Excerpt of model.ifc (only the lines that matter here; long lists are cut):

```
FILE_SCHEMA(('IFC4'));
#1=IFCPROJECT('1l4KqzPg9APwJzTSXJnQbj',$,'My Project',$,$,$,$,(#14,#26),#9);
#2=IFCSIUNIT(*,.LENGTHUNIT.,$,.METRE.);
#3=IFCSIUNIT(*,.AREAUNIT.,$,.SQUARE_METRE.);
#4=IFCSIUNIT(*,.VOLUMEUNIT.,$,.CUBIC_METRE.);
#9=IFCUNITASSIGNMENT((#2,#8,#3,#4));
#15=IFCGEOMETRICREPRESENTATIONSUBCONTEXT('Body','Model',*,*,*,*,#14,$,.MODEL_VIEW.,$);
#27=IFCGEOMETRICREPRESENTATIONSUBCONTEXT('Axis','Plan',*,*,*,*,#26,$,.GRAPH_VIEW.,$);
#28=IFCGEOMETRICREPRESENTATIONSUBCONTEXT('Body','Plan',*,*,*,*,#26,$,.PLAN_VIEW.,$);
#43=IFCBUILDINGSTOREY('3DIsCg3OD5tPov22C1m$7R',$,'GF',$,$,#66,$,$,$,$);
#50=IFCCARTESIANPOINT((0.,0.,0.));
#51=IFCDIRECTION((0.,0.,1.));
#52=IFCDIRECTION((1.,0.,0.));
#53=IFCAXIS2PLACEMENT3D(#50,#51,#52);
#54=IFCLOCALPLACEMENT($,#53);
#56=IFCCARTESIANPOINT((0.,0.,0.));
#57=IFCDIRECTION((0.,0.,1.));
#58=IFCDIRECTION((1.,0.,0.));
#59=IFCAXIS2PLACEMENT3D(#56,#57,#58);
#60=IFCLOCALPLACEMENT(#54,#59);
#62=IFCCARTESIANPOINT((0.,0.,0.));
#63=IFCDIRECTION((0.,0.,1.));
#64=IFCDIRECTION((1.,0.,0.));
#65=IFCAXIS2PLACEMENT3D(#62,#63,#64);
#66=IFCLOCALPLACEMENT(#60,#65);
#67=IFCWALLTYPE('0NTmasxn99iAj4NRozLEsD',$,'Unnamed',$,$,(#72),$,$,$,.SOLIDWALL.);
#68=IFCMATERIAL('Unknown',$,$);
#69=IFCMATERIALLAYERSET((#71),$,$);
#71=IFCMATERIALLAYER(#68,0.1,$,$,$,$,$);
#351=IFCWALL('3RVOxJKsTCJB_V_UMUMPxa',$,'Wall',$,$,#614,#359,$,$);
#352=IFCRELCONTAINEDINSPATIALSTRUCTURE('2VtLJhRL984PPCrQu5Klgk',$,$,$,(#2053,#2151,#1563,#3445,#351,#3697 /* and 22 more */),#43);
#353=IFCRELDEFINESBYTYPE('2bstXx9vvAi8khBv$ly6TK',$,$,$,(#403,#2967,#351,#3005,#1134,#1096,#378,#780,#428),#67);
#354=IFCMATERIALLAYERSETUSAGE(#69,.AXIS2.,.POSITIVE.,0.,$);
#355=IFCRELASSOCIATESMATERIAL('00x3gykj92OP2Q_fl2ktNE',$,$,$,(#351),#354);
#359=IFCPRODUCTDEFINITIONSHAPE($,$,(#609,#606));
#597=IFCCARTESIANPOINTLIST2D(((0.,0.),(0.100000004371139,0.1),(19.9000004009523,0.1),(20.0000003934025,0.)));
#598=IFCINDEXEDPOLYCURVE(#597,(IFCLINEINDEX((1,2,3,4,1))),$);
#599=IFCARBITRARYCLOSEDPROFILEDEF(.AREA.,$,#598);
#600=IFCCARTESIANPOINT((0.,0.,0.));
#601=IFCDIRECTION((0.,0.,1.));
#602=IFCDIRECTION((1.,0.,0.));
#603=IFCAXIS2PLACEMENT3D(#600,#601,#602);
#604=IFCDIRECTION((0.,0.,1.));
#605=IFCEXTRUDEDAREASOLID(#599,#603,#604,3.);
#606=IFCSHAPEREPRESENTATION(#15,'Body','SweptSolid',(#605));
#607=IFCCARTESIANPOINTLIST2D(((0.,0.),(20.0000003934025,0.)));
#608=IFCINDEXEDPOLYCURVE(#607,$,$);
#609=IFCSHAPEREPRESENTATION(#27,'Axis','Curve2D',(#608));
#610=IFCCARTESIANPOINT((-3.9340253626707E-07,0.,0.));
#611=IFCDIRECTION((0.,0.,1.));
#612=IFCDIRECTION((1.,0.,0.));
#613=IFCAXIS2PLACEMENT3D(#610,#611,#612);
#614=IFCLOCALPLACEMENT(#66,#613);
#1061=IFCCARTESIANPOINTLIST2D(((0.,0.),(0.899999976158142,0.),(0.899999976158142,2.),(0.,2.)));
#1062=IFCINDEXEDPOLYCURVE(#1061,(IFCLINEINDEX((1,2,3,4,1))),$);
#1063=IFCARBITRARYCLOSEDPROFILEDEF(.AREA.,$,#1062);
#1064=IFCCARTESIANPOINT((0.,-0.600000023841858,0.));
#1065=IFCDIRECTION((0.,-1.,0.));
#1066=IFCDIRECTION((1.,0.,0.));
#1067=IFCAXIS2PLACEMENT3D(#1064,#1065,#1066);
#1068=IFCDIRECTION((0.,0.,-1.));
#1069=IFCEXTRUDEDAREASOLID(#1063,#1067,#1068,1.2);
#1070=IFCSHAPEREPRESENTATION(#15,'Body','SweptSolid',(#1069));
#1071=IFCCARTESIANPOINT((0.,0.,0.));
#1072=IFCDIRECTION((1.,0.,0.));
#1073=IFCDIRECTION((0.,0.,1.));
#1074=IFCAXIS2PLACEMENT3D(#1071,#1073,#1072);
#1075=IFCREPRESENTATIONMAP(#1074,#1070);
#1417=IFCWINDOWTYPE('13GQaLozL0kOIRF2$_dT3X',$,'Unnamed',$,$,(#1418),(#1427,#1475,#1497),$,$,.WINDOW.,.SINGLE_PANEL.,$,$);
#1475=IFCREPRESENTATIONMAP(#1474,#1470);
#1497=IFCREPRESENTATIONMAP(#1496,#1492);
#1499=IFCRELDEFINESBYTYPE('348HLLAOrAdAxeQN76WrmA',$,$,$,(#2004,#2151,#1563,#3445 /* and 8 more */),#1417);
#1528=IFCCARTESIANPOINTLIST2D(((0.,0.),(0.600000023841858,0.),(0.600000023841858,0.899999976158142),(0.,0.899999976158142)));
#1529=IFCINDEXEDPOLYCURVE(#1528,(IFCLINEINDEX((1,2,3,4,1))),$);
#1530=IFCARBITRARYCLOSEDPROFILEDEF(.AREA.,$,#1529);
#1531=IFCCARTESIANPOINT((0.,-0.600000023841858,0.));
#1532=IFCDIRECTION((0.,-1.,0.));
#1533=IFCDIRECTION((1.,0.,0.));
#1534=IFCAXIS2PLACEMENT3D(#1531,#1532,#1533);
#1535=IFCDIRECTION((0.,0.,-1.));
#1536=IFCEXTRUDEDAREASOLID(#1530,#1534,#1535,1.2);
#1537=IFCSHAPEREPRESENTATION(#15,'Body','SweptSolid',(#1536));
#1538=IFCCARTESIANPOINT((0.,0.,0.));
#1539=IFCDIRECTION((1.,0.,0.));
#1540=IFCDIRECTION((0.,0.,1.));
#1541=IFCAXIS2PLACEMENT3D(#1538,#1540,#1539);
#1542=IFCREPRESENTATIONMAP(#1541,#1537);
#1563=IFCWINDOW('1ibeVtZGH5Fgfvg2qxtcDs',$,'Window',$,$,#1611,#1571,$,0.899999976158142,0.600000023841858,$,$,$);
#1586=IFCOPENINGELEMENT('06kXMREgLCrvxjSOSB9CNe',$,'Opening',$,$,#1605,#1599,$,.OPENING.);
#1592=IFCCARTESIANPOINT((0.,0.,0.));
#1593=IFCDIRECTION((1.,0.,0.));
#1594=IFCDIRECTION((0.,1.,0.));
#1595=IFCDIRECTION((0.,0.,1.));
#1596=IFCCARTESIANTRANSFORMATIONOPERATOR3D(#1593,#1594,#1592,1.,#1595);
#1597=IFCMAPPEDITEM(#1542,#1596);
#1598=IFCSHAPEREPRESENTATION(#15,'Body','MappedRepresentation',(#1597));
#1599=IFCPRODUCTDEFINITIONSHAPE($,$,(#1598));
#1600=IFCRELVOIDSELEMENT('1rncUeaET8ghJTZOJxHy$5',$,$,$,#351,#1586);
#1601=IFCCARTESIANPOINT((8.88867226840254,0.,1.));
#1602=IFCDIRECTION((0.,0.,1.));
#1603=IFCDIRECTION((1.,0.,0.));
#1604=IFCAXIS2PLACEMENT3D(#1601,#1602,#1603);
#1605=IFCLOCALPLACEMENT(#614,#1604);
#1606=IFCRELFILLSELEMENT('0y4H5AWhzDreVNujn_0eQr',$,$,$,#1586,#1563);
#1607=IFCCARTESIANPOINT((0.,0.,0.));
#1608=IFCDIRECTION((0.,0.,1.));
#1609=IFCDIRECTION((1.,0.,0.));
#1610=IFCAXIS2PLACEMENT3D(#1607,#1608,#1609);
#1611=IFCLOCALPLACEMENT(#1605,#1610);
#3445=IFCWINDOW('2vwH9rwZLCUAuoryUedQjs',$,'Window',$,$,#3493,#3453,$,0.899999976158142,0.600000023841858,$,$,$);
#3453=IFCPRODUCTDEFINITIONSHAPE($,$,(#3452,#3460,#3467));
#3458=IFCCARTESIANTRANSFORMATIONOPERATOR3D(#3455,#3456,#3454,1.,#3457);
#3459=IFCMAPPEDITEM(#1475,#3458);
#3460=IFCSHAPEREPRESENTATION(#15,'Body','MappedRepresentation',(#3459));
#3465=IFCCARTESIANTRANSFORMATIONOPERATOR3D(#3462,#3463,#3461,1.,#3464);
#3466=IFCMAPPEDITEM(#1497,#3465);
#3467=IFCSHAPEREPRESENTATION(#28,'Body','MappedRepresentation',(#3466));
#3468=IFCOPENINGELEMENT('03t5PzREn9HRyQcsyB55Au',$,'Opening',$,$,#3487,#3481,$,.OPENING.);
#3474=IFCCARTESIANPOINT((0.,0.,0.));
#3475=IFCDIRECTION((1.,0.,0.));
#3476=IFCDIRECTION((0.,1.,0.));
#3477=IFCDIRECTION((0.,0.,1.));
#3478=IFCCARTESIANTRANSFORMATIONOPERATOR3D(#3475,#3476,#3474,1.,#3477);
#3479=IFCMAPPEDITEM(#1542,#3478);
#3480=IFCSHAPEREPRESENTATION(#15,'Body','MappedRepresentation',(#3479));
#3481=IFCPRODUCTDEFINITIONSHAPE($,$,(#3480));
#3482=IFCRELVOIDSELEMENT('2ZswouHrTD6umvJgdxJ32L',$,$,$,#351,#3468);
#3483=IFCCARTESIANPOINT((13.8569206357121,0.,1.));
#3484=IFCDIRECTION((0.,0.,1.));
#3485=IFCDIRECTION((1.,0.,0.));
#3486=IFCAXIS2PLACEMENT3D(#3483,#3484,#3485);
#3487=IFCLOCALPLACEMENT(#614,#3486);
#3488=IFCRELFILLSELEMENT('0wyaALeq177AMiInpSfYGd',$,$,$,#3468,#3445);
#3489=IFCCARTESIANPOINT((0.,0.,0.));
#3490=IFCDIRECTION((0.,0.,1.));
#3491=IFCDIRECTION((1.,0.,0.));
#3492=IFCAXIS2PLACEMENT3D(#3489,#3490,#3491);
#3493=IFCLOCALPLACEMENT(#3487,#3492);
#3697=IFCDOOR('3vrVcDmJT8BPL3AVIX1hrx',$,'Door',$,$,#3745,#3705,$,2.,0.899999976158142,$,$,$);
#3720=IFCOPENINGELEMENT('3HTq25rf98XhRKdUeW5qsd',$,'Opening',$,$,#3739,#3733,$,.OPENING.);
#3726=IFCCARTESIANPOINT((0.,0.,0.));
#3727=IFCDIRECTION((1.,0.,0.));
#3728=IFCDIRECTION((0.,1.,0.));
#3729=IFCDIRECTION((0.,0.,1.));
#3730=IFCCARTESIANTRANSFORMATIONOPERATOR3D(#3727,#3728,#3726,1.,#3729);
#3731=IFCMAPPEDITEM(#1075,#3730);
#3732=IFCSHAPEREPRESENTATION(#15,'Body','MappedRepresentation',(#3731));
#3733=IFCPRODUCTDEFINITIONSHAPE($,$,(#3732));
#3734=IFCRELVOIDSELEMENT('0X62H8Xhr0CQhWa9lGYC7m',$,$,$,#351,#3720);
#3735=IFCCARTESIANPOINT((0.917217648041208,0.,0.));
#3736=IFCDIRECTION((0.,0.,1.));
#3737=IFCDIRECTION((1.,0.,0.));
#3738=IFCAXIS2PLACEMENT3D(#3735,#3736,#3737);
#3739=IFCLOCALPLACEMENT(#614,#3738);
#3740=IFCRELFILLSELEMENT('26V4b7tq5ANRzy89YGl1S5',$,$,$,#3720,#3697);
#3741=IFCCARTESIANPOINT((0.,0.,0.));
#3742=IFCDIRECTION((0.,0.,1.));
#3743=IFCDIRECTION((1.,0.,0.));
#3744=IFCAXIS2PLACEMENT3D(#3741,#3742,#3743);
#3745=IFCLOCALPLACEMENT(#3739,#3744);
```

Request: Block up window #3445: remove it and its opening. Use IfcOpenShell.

```python
import ifcopenshell
import ifcopenshell.api.feature
import ifcopenshell.api.root
import ifcopenshell.geom
import ifcopenshell.util.shape

model = ifcopenshell.open("model.ifc")
settings = ifcopenshell.geom.settings()


def volume(element):
    """Net volume in cubic metres, openings subtracted."""
    shape = ifcopenshell.geom.create_shape(settings, element)
    return ifcopenshell.util.shape.get_volume(shape.geometry)


window = model.by_guid("2vwH9rwZLCUAuoryUedQjs")
opening = window.FillsVoids[0].RelatingOpeningElement
wall = opening.VoidsElements[0].RelatingBuildingElement
before = volume(wall)

ifcopenshell.api.root.remove_product(model, product=window)
ifcopenshell.api.feature.remove_feature(model, feature=opening)

after = volume(wall)

print(f"wall volume {before:.3f} -> {after:.3f} m3")

model.write("model-out.ifc")
```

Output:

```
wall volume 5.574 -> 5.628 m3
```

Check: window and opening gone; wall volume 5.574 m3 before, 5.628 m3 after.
